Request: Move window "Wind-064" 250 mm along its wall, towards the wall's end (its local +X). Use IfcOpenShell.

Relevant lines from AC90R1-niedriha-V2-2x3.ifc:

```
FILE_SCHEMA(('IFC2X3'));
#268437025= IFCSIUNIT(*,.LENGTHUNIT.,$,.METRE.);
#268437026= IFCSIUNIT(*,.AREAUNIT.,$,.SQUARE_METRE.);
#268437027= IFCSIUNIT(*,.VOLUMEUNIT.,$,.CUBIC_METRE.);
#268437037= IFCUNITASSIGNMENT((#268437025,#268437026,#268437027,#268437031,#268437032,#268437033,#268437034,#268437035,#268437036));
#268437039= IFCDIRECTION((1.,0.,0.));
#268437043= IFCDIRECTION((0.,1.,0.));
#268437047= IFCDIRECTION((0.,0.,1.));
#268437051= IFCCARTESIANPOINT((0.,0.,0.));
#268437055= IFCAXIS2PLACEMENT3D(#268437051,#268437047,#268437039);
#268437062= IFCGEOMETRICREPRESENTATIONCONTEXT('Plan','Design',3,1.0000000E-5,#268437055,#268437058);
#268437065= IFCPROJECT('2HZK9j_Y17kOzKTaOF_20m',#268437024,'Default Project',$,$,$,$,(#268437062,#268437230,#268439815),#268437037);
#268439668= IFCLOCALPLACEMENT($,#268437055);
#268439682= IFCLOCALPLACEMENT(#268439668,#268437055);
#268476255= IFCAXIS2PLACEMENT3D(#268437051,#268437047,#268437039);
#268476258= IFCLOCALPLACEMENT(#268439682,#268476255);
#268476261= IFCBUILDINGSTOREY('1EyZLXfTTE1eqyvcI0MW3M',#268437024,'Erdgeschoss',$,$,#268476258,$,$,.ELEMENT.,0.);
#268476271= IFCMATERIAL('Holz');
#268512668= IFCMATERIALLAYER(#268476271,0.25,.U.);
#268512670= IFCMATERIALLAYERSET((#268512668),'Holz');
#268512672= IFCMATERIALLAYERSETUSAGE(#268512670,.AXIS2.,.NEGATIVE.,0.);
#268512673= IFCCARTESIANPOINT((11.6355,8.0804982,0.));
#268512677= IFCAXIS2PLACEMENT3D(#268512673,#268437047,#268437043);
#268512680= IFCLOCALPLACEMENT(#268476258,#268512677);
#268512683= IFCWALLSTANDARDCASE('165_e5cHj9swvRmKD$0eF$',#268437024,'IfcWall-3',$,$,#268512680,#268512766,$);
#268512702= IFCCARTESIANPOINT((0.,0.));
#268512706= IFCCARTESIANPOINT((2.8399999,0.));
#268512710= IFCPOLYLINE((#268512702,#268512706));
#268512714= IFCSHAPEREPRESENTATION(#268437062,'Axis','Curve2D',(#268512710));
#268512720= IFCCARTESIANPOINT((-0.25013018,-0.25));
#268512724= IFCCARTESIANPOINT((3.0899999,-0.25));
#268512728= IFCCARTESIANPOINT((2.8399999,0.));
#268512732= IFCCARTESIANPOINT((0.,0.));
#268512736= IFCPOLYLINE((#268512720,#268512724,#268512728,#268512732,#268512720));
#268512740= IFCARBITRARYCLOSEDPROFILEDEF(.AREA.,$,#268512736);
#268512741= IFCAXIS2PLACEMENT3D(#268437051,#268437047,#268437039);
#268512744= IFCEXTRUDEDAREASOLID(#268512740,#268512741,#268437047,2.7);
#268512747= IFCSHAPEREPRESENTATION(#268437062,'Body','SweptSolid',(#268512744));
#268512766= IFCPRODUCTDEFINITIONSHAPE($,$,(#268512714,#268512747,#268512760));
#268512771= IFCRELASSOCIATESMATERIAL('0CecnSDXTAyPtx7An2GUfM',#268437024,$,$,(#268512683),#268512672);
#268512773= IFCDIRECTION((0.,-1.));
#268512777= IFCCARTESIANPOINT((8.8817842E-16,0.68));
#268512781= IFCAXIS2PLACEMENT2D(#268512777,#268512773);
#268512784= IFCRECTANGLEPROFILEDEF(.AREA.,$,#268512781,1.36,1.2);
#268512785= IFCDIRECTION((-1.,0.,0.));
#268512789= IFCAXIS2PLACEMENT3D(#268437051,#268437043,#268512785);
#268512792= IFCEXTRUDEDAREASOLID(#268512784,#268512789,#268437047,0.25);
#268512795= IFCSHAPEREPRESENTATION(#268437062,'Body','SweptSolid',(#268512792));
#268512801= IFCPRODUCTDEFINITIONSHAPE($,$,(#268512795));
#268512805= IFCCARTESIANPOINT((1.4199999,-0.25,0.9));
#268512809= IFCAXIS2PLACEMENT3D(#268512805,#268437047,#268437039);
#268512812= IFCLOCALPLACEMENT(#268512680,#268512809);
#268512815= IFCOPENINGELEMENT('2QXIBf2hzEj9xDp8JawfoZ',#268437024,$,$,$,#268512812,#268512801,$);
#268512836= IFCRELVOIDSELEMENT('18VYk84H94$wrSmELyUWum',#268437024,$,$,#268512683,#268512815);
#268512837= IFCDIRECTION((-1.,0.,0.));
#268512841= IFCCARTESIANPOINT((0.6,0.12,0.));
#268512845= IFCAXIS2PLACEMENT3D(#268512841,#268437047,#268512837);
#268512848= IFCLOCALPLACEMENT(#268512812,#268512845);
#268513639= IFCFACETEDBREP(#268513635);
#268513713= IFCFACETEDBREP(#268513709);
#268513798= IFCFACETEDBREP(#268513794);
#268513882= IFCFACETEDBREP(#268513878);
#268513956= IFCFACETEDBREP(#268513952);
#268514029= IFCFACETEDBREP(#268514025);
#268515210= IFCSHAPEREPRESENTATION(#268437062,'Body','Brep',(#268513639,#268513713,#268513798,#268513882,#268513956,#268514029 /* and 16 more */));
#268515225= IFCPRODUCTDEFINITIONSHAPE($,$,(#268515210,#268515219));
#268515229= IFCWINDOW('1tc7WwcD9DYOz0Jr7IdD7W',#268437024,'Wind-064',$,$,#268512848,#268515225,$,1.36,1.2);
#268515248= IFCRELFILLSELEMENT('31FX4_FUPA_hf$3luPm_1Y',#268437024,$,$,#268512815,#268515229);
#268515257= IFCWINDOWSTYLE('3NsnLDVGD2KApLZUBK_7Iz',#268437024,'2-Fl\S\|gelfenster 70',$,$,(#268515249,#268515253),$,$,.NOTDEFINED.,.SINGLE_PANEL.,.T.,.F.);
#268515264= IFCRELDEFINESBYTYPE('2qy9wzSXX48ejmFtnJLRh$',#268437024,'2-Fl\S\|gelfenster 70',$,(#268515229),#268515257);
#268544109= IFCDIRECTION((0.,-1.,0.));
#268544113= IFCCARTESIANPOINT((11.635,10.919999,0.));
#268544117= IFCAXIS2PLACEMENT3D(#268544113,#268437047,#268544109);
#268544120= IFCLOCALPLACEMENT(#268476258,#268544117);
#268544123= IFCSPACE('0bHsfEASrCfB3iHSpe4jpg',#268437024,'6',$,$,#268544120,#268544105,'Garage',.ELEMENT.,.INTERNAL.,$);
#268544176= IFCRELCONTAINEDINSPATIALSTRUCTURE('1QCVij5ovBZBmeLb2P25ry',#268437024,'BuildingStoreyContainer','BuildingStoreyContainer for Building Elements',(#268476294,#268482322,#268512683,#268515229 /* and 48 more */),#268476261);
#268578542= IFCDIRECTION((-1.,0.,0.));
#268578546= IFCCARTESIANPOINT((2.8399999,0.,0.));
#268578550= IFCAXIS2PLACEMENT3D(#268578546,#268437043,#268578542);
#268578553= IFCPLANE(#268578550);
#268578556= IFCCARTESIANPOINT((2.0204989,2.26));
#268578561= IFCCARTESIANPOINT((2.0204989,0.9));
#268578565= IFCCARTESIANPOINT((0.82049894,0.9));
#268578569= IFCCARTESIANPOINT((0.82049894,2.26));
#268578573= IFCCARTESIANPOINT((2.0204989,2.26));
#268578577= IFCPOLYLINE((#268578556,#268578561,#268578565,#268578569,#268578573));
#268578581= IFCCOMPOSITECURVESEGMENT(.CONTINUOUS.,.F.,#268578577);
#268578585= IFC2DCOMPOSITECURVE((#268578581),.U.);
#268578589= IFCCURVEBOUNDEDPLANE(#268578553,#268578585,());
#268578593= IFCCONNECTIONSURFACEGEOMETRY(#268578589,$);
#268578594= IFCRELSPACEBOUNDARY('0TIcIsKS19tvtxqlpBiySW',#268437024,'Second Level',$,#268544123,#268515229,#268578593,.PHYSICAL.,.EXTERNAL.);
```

```python
import numpy as np
import ifcopenshell
import ifcopenshell.api.geometry
import ifcopenshell.util.placement

model = ifcopenshell.open("AC90R1-niedriha-V2-2x3.ifc")

window = model.by_id(268515229)
opening = window.FillsVoids[0].RelatingOpeningElement
wall = opening.VoidsElements[0].RelatingBuildingElement

wall_matrix = ifcopenshell.util.placement.get_local_placement(wall.ObjectPlacement)
shift = wall_matrix[:3, 0] * 0.25
before = ifcopenshell.util.placement.get_local_placement(window.ObjectPlacement)[:3, 3].copy()

# The window is placed relative to its opening, so it follows when the opening moves.
matrix = ifcopenshell.util.placement.get_local_placement(opening.ObjectPlacement)
matrix[:3, 3] += shift
ifcopenshell.api.geometry.edit_object_placement(
    model, product=opening, matrix=matrix, is_si=False, should_transform_children=True
)

# Space boundary surfaces are stored in each space's coordinates; move them too.
for rel in window.ProvidesBoundaries:
    if not rel.ConnectionGeometry:
        continue
    surface = rel.ConnectionGeometry.SurfaceOnRelatingElement.BasisSurface
    space_matrix = ifcopenshell.util.placement.get_local_placement(rel.RelatingSpace.ObjectPlacement)
    point = np.array(surface.Position.Location.Coordinates) + space_matrix[:3, :3].T @ shift
    surface.Position = model.createIfcAxis2Placement3D(
        model.createIfcCartesianPoint(point.tolist()), surface.Position.Axis, surface.Position.RefDirection
    )

after = ifcopenshell.util.placement.get_local_placement(window.ObjectPlacement)[:3, 3]
print("window moved by", (after - before).round(3) + 0.0)

model.write("AC90R1-niedriha-V2-2x3_rev.ifc")
```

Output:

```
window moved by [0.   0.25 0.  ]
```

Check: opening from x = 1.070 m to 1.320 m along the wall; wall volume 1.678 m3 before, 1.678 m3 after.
